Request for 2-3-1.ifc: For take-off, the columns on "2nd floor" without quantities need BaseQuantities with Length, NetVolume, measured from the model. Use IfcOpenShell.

First a look at what the model holds.

```python
import ifcopenshell
import ifcopenshell.util.element
import ifcopenshell.util.unit

model = ifcopenshell.open("2-3-1.ifc")
print(model.schema)
for unit_type in ("LENGTHUNIT", "AREAUNIT", "VOLUMEUNIT"):
    print(unit_type, ifcopenshell.util.unit.calculate_unit_scale(model, unit_type))
storey = next(s for s in model.by_type("IfcBuildingStorey") if s.Name == "2nd floor")
columns = [e for e in ifcopenshell.util.element.get_decomposition(storey) if e.is_a("IfcColumn")]
for e in sorted(columns, key=lambda e: e.id()):
    print(e.id(), e.is_a(), e.Name, list(ifcopenshell.util.element.get_psets(e, qtos_only=True)), sep=" | ")
```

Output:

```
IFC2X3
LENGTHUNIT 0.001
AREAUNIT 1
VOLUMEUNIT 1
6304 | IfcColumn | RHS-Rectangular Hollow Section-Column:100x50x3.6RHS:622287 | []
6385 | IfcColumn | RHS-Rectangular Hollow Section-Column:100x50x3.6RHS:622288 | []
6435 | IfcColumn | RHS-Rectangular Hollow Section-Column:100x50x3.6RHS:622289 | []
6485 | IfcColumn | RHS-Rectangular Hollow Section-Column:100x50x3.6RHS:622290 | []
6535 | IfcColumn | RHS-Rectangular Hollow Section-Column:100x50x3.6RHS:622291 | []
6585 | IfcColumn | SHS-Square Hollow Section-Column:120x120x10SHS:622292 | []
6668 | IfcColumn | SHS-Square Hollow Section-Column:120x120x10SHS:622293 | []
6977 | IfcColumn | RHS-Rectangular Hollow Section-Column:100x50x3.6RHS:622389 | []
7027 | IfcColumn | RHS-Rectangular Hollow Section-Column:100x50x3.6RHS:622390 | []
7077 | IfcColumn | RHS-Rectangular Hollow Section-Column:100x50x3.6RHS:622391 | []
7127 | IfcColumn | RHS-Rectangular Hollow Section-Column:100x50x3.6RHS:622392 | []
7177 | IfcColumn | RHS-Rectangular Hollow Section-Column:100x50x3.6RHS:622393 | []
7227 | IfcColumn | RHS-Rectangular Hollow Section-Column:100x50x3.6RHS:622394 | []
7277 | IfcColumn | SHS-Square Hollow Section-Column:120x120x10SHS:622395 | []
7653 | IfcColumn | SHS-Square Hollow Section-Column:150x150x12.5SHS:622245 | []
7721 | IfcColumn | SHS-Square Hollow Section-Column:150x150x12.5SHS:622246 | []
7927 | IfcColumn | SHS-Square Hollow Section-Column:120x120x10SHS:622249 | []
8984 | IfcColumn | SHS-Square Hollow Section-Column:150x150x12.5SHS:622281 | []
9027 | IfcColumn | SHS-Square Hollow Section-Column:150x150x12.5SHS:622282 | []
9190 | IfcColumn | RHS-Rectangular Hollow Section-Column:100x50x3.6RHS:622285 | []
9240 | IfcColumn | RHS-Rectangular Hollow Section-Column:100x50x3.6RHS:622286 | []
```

```python
import ifcopenshell
import ifcopenshell.api.pset
import ifcopenshell.geom
import ifcopenshell.util.element
import ifcopenshell.util.shape
import ifcopenshell.util.unit

model = ifcopenshell.open("2-3-1.ifc")
unit_scale = ifcopenshell.util.unit.calculate_unit_scale(model)
volume_scale = ifcopenshell.util.unit.calculate_unit_scale(model, "VOLUMEUNIT")
settings = ifcopenshell.geom.settings()

storey = next(s for s in model.by_type("IfcBuildingStorey") if s.Name == "2nd floor")
columns = [e for e in ifcopenshell.util.element.get_decomposition(storey) if e.is_a("IfcColumn")]

for e in sorted(columns, key=lambda e: e.id()):
    if ifcopenshell.util.element.get_psets(e, qtos_only=True, should_inherit=False):
        continue
    # Geometry comes back in metres, in the element's own axes.
    shape = ifcopenshell.geom.create_shape(settings, e)
    values = {
        "Length": ifcopenshell.util.shape.get_z(shape.geometry) / unit_scale,
        "NetVolume": ifcopenshell.util.shape.get_volume(shape.geometry) / volume_scale,
    }
    qto = ifcopenshell.api.pset.add_qto(model, product=e, name="BaseQuantities")
    ifcopenshell.api.pset.edit_qto(model, qto=qto, properties=values)
    print(e.id(), {k: round(v, 3) for k, v in values.items()})

model.write("2-3-1-out.ifc")
```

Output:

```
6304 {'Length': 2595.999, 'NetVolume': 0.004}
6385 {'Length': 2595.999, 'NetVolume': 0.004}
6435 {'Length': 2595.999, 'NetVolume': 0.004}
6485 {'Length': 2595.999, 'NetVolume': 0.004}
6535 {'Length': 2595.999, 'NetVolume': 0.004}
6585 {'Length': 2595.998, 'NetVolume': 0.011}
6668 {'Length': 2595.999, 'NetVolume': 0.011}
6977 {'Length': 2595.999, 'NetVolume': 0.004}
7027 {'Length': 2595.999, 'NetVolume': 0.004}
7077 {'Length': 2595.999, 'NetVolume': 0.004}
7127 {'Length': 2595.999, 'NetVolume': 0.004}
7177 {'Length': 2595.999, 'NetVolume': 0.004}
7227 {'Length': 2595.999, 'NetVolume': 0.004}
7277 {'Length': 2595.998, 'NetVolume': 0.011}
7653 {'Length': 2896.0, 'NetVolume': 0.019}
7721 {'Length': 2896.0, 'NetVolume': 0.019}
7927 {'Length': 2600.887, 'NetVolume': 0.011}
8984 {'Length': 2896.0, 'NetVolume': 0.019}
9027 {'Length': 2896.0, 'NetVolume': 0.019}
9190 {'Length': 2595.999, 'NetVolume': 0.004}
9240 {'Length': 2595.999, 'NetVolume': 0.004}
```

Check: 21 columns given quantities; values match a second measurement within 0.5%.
